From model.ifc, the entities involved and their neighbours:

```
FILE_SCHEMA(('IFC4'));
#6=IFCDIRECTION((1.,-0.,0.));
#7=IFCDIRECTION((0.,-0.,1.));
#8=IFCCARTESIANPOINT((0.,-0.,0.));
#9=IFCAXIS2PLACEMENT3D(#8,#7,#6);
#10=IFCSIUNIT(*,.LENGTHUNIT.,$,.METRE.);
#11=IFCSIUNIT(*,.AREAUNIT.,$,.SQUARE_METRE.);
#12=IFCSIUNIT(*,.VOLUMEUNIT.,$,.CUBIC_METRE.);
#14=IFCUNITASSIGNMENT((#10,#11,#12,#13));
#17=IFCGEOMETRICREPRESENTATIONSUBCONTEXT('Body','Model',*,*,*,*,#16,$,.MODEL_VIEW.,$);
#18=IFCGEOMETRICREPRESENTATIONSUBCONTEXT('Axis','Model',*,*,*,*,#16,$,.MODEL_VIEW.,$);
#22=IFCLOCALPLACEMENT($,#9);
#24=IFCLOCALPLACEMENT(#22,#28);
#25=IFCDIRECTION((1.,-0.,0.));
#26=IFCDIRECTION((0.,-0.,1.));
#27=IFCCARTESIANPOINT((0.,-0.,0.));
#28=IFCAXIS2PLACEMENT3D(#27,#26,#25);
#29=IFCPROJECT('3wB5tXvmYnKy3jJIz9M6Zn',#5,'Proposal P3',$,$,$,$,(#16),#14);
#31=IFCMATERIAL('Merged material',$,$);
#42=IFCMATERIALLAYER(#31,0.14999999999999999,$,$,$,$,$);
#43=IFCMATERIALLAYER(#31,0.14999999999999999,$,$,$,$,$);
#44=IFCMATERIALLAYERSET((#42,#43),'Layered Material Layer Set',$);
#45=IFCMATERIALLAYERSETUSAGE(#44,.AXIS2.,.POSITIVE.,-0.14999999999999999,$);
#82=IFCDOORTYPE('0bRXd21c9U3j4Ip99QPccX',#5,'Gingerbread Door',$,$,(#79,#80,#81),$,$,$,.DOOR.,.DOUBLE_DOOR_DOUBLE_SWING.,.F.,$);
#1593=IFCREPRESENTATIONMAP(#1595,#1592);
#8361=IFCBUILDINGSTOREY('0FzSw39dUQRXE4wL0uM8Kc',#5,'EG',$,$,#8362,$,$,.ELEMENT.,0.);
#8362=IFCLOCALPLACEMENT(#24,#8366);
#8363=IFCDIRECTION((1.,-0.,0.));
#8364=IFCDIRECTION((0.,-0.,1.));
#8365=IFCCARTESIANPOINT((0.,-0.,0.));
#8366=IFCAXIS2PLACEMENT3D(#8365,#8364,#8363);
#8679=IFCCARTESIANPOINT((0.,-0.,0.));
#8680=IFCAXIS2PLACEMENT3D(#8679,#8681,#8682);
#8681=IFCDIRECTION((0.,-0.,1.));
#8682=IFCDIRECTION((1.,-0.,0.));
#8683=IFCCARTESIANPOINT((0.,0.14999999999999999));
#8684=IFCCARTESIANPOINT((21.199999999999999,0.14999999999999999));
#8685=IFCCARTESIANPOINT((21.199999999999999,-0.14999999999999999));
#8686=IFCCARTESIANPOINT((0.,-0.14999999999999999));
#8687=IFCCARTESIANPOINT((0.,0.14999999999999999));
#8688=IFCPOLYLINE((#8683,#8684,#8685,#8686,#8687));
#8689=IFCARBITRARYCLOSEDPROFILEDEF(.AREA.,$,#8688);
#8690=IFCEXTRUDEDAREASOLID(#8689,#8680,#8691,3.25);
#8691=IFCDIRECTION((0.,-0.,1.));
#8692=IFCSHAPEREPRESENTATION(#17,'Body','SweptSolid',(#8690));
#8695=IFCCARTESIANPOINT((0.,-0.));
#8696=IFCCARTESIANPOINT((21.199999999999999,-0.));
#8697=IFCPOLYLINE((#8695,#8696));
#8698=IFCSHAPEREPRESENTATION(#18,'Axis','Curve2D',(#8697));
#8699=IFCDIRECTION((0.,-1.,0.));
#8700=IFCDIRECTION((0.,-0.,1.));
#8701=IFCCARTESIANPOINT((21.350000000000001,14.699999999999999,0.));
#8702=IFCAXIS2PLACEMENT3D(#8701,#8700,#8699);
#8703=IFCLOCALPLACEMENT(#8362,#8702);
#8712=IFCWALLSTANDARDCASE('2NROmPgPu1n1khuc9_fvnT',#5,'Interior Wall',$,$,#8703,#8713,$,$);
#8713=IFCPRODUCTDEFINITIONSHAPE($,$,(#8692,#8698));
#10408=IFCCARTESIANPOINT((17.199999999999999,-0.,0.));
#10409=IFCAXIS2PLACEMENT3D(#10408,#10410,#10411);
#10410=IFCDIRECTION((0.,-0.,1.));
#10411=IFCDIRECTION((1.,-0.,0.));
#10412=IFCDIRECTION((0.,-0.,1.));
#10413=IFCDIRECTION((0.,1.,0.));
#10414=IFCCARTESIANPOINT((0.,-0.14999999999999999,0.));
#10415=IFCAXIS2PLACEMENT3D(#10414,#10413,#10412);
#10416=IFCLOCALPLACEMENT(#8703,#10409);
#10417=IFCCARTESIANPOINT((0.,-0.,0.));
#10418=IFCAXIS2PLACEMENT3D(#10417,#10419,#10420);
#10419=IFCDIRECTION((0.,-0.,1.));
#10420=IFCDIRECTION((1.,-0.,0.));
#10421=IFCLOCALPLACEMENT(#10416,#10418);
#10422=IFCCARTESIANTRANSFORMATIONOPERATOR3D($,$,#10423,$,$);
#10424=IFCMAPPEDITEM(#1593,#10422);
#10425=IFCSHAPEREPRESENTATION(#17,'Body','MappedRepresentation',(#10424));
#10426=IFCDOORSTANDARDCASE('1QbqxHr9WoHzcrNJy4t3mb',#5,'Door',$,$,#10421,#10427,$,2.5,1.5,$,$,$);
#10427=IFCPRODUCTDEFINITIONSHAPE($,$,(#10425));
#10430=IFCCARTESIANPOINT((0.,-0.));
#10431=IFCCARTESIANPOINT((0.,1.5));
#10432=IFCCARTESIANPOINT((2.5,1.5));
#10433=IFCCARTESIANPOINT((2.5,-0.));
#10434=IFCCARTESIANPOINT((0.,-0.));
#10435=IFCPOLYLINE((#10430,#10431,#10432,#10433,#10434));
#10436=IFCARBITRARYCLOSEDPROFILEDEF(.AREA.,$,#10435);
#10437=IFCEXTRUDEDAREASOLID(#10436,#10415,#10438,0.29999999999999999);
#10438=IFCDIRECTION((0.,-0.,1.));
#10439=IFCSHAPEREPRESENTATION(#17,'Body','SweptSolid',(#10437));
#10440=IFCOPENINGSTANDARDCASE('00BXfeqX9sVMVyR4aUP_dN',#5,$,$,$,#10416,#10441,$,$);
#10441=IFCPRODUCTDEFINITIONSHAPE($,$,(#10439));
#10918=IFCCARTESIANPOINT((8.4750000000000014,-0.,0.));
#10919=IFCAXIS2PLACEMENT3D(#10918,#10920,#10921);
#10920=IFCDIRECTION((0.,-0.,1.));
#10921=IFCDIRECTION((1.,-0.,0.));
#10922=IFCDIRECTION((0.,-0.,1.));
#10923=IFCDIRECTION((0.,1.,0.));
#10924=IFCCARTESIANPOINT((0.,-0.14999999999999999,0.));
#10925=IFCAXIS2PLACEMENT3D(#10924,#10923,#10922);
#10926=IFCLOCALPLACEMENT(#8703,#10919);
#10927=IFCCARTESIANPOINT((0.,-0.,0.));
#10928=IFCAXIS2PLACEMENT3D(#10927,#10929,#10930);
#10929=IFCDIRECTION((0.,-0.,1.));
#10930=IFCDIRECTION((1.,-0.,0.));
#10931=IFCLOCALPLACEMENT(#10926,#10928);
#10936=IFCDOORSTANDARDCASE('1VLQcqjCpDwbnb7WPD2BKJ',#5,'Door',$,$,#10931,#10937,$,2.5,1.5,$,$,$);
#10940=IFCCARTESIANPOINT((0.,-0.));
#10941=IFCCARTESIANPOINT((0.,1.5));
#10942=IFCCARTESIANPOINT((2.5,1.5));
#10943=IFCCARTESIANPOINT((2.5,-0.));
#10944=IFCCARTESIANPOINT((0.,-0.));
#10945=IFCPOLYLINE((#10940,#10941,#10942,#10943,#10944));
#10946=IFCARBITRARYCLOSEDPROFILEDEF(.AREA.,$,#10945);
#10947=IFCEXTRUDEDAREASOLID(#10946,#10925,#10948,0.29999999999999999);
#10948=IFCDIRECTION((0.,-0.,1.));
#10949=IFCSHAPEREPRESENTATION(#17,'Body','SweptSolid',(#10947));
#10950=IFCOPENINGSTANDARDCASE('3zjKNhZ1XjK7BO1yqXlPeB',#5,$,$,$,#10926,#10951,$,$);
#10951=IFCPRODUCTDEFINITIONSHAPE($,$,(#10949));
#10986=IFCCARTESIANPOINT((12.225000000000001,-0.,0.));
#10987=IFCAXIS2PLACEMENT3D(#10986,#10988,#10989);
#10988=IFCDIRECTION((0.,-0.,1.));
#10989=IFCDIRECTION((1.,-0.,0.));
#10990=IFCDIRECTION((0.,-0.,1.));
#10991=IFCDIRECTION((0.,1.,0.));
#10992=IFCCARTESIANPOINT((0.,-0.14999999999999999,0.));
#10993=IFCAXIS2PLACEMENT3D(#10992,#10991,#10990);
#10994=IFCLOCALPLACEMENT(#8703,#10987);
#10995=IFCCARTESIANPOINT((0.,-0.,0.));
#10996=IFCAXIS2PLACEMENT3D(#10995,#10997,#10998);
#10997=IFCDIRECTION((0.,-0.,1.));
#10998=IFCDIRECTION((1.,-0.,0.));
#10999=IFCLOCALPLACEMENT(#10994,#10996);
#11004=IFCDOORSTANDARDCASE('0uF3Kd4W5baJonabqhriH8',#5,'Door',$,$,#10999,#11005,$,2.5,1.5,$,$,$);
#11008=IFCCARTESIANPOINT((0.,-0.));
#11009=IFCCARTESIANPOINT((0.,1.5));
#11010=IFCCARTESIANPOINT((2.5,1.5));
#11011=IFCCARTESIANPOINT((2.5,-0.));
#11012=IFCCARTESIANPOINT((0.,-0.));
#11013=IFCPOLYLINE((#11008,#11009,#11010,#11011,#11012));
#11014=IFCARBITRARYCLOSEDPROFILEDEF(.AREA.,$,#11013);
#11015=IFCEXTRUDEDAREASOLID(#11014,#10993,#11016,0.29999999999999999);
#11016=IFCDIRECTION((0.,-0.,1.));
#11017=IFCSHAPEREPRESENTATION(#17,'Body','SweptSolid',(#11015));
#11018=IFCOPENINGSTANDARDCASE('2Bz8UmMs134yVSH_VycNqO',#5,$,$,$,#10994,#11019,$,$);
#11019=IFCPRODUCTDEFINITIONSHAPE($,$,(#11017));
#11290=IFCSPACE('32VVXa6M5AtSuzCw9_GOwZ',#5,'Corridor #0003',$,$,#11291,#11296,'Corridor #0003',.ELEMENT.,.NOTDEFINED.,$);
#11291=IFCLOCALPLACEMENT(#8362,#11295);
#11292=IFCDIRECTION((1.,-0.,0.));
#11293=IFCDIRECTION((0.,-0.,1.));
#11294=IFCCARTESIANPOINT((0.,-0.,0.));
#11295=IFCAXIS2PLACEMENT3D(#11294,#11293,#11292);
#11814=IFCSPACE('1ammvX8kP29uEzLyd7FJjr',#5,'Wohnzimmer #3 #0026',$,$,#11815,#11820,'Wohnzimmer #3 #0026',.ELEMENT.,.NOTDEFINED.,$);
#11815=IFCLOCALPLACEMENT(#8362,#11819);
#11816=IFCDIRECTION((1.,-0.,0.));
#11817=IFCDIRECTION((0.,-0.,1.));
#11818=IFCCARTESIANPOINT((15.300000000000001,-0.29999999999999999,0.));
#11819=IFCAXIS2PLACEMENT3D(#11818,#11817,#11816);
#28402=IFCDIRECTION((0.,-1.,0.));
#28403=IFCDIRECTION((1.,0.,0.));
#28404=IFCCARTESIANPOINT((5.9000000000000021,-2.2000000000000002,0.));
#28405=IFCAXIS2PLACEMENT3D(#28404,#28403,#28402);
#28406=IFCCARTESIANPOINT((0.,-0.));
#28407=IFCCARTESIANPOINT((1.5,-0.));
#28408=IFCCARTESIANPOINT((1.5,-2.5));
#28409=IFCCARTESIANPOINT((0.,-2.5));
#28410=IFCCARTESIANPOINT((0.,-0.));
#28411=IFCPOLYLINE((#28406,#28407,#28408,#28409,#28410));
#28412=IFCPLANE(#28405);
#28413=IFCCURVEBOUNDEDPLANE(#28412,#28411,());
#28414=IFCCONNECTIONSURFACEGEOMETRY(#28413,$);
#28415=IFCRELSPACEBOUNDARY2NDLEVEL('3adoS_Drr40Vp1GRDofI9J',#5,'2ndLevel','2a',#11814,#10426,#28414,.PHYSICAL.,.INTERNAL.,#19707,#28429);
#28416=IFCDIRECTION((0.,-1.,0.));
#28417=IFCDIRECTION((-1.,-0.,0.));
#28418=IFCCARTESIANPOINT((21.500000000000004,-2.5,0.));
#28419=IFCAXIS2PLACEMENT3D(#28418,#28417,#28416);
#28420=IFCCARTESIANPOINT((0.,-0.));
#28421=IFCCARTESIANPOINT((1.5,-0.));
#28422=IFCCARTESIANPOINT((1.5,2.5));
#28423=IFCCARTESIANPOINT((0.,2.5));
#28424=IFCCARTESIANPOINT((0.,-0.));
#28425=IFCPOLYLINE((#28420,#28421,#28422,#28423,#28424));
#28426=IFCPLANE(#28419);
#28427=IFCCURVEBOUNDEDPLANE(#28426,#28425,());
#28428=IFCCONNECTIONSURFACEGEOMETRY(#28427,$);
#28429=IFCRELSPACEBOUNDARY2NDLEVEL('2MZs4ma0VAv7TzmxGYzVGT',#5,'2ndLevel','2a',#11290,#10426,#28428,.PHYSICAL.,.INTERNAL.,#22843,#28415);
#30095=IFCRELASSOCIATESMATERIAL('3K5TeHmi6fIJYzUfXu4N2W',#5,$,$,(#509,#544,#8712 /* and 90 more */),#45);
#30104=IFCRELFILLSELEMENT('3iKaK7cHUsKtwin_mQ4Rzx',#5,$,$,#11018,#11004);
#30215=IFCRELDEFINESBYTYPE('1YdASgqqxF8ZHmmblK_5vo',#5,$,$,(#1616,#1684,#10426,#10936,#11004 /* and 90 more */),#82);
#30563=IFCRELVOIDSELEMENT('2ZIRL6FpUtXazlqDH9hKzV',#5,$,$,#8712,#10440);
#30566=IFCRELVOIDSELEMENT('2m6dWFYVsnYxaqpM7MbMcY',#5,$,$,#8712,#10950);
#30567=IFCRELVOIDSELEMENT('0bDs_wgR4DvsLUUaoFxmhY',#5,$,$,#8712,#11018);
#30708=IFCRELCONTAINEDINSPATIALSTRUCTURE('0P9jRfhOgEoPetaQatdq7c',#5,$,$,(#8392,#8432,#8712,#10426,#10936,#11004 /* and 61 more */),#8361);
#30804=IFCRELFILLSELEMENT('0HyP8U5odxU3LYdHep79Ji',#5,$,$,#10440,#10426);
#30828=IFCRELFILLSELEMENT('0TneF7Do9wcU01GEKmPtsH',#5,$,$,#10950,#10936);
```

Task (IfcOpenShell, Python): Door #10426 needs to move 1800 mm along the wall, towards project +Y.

```python
import numpy as np
import ifcopenshell
import ifcopenshell.api.geometry
import ifcopenshell.util.placement
import ifcopenshell.util.unit

model = ifcopenshell.open("model.ifc")
unit_scale = ifcopenshell.util.unit.calculate_unit_scale(model)

door = model.by_id(10426)
opening = door.FillsVoids[0].RelatingOpeningElement
wall = opening.VoidsElements[0].RelatingBuildingElement

wall_matrix = ifcopenshell.util.placement.get_local_placement(wall.ObjectPlacement)
shift = wall_matrix[:3, 0] * -1.8 / unit_scale
before = ifcopenshell.util.placement.get_local_placement(door.ObjectPlacement)[:3, 3].copy()

# The door is placed relative to its opening, so it follows when the opening moves.
matrix = ifcopenshell.util.placement.get_local_placement(opening.ObjectPlacement)
matrix[:3, 3] += shift
ifcopenshell.api.geometry.edit_object_placement(
    model, product=opening, matrix=matrix, is_si=False, should_transform_children=True
)

# Space boundary surfaces are stored in each space's coordinates; move them too.
for rel in door.ProvidesBoundaries:
    if not rel.ConnectionGeometry:
        continue
    surface = rel.ConnectionGeometry.SurfaceOnRelatingElement.BasisSurface
    space_matrix = ifcopenshell.util.placement.get_local_placement(rel.RelatingSpace.ObjectPlacement)
    point = np.array(surface.Position.Location.Coordinates) + space_matrix[:3, :3].T @ shift
    surface.Position = model.createIfcAxis2Placement3D(
        model.createIfcCartesianPoint(point.tolist()), surface.Position.Axis, surface.Position.RefDirection
    )

after = ifcopenshell.util.placement.get_local_placement(door.ObjectPlacement)[:3, 3]
print("door moved by", (after - before).round(3) + 0.0)

model.write("model_rev.ifc")
```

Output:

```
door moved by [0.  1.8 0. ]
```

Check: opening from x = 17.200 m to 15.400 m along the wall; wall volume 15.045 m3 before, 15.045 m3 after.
